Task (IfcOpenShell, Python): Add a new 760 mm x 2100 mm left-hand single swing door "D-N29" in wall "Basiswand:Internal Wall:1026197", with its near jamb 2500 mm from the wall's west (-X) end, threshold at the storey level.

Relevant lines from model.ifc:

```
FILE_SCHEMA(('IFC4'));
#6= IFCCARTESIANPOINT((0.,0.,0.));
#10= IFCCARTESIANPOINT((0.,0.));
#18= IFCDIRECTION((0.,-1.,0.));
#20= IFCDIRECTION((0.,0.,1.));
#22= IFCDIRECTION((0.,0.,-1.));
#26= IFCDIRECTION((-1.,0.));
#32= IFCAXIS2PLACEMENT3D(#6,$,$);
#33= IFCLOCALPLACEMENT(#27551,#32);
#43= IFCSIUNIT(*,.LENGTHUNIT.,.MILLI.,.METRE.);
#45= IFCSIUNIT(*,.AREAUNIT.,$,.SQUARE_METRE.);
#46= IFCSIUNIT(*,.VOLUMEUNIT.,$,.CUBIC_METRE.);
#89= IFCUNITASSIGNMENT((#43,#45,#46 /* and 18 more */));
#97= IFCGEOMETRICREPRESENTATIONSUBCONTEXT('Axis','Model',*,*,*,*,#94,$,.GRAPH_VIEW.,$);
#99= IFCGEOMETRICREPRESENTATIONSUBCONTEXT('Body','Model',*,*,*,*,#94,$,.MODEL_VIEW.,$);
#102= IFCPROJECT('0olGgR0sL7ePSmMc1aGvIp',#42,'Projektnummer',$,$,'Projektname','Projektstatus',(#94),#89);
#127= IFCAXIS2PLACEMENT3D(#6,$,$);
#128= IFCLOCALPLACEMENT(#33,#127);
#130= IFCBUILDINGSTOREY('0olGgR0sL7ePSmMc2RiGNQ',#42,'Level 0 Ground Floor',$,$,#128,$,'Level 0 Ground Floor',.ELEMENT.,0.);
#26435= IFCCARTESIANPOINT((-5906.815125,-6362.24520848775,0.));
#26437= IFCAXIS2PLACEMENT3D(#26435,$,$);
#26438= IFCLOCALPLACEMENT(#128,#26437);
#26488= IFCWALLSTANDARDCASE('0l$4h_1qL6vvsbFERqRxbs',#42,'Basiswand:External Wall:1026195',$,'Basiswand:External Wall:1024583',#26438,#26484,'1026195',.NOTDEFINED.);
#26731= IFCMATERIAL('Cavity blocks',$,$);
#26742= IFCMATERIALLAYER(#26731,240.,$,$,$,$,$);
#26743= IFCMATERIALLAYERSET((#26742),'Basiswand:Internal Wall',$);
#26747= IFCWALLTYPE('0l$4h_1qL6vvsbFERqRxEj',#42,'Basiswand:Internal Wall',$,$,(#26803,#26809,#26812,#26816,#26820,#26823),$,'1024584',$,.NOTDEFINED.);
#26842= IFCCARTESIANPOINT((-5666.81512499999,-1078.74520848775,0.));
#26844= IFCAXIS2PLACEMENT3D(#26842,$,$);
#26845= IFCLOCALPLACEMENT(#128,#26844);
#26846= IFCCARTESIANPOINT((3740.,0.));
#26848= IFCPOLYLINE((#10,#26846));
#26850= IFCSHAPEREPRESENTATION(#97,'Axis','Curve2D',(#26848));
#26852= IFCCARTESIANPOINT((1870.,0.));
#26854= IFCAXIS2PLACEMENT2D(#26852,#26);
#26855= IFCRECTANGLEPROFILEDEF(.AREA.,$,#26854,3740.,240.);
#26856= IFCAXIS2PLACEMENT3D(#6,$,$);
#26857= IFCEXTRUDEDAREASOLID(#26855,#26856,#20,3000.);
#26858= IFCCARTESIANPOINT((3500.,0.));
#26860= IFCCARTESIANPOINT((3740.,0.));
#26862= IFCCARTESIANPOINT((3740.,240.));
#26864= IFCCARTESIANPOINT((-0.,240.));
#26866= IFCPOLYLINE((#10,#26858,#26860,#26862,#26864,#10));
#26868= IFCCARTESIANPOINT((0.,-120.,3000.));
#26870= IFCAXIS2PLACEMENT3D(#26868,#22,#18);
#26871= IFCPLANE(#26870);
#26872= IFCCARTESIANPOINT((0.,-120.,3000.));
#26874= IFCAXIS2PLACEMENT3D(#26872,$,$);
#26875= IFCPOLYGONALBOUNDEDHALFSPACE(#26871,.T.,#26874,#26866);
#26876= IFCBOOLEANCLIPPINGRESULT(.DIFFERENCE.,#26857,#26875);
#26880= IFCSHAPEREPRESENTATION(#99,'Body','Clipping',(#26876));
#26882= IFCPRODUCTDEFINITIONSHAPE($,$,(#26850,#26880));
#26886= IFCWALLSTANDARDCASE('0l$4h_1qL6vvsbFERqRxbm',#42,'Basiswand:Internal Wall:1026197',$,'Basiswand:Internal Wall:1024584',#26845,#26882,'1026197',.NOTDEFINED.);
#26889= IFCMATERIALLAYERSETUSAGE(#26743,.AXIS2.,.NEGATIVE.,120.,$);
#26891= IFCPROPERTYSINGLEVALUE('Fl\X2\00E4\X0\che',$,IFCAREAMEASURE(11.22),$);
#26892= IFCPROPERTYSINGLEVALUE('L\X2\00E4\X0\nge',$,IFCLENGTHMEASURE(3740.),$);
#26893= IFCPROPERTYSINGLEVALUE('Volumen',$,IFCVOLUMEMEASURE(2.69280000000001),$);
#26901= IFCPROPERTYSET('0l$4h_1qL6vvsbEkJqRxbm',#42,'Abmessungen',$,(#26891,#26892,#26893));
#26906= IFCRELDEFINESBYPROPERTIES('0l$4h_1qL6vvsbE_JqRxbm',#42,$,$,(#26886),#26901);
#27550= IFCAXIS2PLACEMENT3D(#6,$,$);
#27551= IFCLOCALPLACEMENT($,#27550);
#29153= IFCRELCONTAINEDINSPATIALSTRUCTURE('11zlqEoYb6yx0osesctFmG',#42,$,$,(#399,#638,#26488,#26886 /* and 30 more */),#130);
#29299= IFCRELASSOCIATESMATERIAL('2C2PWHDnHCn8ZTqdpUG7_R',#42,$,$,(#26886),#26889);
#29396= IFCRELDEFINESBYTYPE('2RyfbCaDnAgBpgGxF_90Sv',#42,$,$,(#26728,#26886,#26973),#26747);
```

```python
import numpy as np
import ifcopenshell
import ifcopenshell.api.feature
import ifcopenshell.api.geometry
import ifcopenshell.api.pset
import ifcopenshell.api.root
import ifcopenshell.api.spatial
import ifcopenshell.geom
import ifcopenshell.util.element
import ifcopenshell.util.placement
import ifcopenshell.util.representation
import ifcopenshell.util.shape
import ifcopenshell.util.unit

model = ifcopenshell.open("model.ifc")
unit_scale = ifcopenshell.util.unit.calculate_unit_scale(model)
area_scale = ifcopenshell.util.unit.calculate_unit_scale(model, "AREAUNIT")
volume_scale = ifcopenshell.util.unit.calculate_unit_scale(model, "VOLUMEUNIT")
settings = ifcopenshell.geom.settings()


def volume(element):
    """Net volume in cubic metres, openings subtracted."""
    shape = ifcopenshell.geom.create_shape(settings, element)
    return ifcopenshell.util.shape.get_volume(shape.geometry)


wall = model.by_id(26886)
storey = ifcopenshell.util.element.get_container(wall, ifc_class="IfcBuildingStorey")
context = ifcopenshell.util.representation.get_context(model, "Model", "Body", "MODEL_VIEW")
before = volume(wall)

width, height, from_end, sill = 0.76, 2.1, 2.5, 0.0  # metres

# The wall runs along its own X axis, and the end named is its -X end.
wall_shape = ifcopenshell.geom.create_shape(settings, wall)
x, y, z = ifcopenshell.util.shape.get_vertices(wall_shape.geometry).T
start = x.min() + from_end
face, thickness = float(y.min()), float(y.max() - y.min())
wall_matrix = ifcopenshell.util.placement.get_local_placement(wall.ObjectPlacement)
level = ifcopenshell.util.placement.get_local_placement(storey.ObjectPlacement)[2, 3]


def in_wall(x, y):
    """Placement at x, y metres in the wall's axes, at sill height."""
    matrix = wall_matrix.copy()
    matrix[:, 3] = wall_matrix @ np.array([x / unit_scale, y / unit_scale, 0.0, 1.0])
    matrix[2, 3] = level + sill / unit_scale
    return matrix


# Opening: a box that overshoots both wall faces by 50 mm.
opening = ifcopenshell.api.root.create_entity(model, ifc_class="IfcOpeningElement", predefined_type="OPENING")
box = ifcopenshell.api.geometry.add_wall_representation(
    model, context=context, length=width, height=height, thickness=thickness + 0.1
)
ifcopenshell.api.geometry.assign_representation(model, product=opening, representation=box)
ifcopenshell.api.geometry.edit_object_placement(model, product=opening, matrix=in_wall(start, face - 0.05), is_si=False)
ifcopenshell.api.feature.add_feature(model, feature=opening, element=wall)

door = ifcopenshell.api.root.create_entity(model, ifc_class="IfcDoor", name="D-N29", predefined_type="DOOR")
door.OverallWidth, door.OverallHeight = width / unit_scale, height / unit_scale
door.OperationType = "SINGLE_SWING_LEFT"
body = ifcopenshell.api.geometry.add_door_representation(
    model,
    context=context,
    overall_width=door.OverallWidth,
    overall_height=door.OverallHeight,
    operation_type="SINGLE_SWING_LEFT",
    lining_properties={"LiningDepth": thickness / unit_scale, "ThresholdDepth": thickness / unit_scale},
)
ifcopenshell.api.geometry.assign_representation(model, product=door, representation=body)
ifcopenshell.api.spatial.assign_container(model, products=[door], relating_structure=storey)
ifcopenshell.api.feature.add_filling(model, opening=opening, element=door)

# The lining spans the wall, so the door starts at the wall face.
ifcopenshell.api.geometry.edit_object_placement(model, product=door, matrix=in_wall(start, face), is_si=False)

after = volume(wall)

# Update the wall's stored quantities.
pset = model.by_id(ifcopenshell.util.element.get_pset(wall, "Abmessungen", should_inherit=False)["id"])
ifcopenshell.api.pset.edit_pset(model, pset=pset, properties={
    "Fläche": model.create_entity("IfcAreaMeasure", after / thickness / area_scale),
    "Volumen": model.create_entity("IfcVolumeMeasure", after / volume_scale),
})

print(f"wall volume {before:.3f} -> {after:.3f} m3")

model.write("model_updated.ifc")
```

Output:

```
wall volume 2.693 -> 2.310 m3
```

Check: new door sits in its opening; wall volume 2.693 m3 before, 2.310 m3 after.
